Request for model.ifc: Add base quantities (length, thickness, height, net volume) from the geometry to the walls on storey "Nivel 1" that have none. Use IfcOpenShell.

First a look at what the model holds.

```python
import ifcopenshell
import ifcopenshell.util.element
import ifcopenshell.util.unit

model = ifcopenshell.open("model.ifc")
print(model.schema)
for unit_type in ("LENGTHUNIT", "AREAUNIT", "VOLUMEUNIT"):
    print(unit_type, ifcopenshell.util.unit.calculate_unit_scale(model, unit_type))
storey = next(s for s in model.by_type("IfcBuildingStorey") if s.Name == "Nivel 1")
walls = [e for e in ifcopenshell.util.element.get_decomposition(storey) if e.is_a("IfcWall")]
for e in sorted(walls, key=lambda e: e.id()):
    print(e.id(), e.is_a(), e.Name, list(ifcopenshell.util.element.get_psets(e, qtos_only=True)), sep=" | ")
```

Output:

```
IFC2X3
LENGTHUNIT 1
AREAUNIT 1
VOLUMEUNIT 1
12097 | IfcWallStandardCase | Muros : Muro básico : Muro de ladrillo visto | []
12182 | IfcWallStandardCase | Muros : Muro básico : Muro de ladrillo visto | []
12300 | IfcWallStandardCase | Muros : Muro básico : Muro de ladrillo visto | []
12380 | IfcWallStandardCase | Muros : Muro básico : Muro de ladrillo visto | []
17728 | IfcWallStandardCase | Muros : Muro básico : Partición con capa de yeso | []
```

```python
import ifcopenshell
import ifcopenshell.api.pset
import ifcopenshell.geom
import ifcopenshell.util.element
import ifcopenshell.util.shape
import ifcopenshell.util.unit

model = ifcopenshell.open("model.ifc")
unit_scale = ifcopenshell.util.unit.calculate_unit_scale(model)
volume_scale = ifcopenshell.util.unit.calculate_unit_scale(model, "VOLUMEUNIT")
settings = ifcopenshell.geom.settings()

storey = next(s for s in model.by_type("IfcBuildingStorey") if s.Name == "Nivel 1")
walls = [e for e in ifcopenshell.util.element.get_decomposition(storey) if e.is_a("IfcWall")]

for e in sorted(walls, key=lambda e: e.id()):
    if ifcopenshell.util.element.get_psets(e, qtos_only=True, should_inherit=False):
        continue
    # Geometry comes back in metres, in the element's own axes.
    shape = ifcopenshell.geom.create_shape(settings, e)
    values = {
        "Length": ifcopenshell.util.shape.get_x(shape.geometry) / unit_scale,
        "Width": ifcopenshell.util.shape.get_y(shape.geometry) / unit_scale,
        "Height": ifcopenshell.util.shape.get_z(shape.geometry) / unit_scale,
        "NetVolume": ifcopenshell.util.shape.get_volume(shape.geometry) / volume_scale,
    }
    qto = ifcopenshell.api.pset.add_qto(model, product=e, name="BaseQuantities")
    ifcopenshell.api.pset.edit_qto(model, qto=qto, properties=values)
    print(e.id(), {k: round(v, 3) for k, v in values.items()})

model.write("model_rev.ifc")
```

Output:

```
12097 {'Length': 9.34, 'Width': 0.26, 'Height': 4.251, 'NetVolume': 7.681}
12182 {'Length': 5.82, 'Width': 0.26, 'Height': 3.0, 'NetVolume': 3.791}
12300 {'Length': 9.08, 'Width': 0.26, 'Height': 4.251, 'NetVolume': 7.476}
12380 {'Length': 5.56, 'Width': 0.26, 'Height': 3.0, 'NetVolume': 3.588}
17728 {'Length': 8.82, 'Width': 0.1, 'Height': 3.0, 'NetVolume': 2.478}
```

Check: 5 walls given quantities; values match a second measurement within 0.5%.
